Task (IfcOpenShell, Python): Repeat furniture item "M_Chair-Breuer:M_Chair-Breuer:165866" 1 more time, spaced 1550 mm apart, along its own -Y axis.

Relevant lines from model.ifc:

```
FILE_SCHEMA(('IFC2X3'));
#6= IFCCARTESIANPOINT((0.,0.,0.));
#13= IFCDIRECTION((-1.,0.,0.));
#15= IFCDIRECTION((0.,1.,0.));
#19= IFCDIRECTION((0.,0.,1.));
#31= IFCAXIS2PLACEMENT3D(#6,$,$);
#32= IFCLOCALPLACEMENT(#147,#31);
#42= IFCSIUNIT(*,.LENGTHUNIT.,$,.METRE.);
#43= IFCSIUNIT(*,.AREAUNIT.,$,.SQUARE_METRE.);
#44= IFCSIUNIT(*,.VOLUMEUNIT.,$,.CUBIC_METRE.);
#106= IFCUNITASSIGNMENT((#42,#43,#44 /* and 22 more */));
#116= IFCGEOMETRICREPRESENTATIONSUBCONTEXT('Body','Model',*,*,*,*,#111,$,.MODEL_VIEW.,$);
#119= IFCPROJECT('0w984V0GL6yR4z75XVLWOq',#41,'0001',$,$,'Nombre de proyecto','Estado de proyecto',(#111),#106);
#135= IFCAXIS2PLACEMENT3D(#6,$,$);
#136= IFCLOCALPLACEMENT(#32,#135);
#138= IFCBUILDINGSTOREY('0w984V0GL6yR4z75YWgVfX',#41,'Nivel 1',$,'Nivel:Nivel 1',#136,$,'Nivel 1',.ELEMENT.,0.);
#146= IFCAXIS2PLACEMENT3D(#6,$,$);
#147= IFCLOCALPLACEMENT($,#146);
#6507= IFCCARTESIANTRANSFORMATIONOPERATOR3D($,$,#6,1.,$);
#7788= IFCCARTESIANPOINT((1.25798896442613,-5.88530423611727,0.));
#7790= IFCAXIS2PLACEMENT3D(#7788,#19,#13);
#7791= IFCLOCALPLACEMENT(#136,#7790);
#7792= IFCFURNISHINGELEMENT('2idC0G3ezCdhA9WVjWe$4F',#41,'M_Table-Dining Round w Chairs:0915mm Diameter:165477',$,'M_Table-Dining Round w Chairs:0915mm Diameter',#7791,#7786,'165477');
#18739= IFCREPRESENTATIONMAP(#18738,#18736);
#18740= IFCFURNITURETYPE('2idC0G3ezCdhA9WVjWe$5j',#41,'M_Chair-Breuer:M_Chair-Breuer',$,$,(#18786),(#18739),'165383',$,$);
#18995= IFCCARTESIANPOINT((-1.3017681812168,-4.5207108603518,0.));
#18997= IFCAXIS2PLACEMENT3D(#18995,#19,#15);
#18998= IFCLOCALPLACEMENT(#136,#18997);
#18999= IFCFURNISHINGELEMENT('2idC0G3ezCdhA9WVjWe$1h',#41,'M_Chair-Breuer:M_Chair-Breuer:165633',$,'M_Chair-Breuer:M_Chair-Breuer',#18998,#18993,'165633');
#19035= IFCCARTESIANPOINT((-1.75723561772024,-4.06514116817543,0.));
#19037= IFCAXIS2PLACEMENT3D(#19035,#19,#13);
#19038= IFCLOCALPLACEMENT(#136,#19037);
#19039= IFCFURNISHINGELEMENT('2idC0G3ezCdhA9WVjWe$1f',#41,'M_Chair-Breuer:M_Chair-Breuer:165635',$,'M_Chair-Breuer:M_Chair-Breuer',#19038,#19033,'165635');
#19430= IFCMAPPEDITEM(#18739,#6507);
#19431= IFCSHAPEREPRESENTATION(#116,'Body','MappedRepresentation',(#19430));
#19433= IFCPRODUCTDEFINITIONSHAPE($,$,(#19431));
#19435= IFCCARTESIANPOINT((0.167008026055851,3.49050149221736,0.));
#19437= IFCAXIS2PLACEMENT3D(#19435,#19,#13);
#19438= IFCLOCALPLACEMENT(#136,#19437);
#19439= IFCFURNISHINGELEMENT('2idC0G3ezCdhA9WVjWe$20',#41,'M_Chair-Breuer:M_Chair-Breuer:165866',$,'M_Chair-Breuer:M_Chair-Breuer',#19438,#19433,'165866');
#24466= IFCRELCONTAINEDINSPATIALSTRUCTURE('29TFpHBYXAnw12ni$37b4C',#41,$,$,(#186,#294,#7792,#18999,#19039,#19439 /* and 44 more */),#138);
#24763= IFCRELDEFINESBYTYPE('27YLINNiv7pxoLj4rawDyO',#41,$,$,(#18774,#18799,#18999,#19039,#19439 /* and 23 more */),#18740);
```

```python
import ifcopenshell
import ifcopenshell.api.geometry
import ifcopenshell.api.root
import ifcopenshell.util.element
import ifcopenshell.util.placement

model = ifcopenshell.open("model.ifc")


def reuse_history(source, copy):
    """copy_class also copies each property set's owner history, people and application; keep the originals."""
    for rel in copy.IsDefinedBy:
        if rel.is_a("IfcRelDefinesByProperties") and (history := rel.RelatingPropertyDefinition.OwnerHistory):
            rel.RelatingPropertyDefinition.OwnerHistory = source.OwnerHistory
            ifcopenshell.util.element.remove_deep2(model, history)


source = model.by_guid("2idC0G3ezCdhA9WVjWe$20")
base = ifcopenshell.util.placement.get_local_placement(source.ObjectPlacement)
step = -base[:3, 1] * 1.55

for i in range(1, 2):
    copy = ifcopenshell.api.root.copy_class(model, product=source)
    copy.Representation = ifcopenshell.util.element.copy_deep(
        model, source.Representation, exclude=["IfcGeometricRepresentationContext", "IfcRepresentationMap"]
    )
    copy.Name = "M_Chair-Breuer:M_Chair-Breuer"
    copy.Tag = None
    reuse_history(source, copy)
    matrix = base.copy()
    matrix[:3, 3] += i * step
    print("added at", matrix[:3, 3].round(3) + 0.0)
    ifcopenshell.api.geometry.edit_object_placement(model, product=copy, matrix=matrix, is_si=False)

model.write("model_v2.ifc")
```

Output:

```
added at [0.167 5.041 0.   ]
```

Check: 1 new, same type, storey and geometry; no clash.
